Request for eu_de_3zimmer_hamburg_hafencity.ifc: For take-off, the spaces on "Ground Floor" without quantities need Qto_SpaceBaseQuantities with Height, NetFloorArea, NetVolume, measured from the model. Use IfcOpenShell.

First a look at what the model holds.

```python
import ifcopenshell
import ifcopenshell.util.element
import ifcopenshell.util.unit

model = ifcopenshell.open("eu_de_3zimmer_hamburg_hafencity.ifc")
print(model.schema)
for unit_type in ("LENGTHUNIT", "AREAUNIT", "VOLUMEUNIT"):
    print(unit_type, ifcopenshell.util.unit.calculate_unit_scale(model, unit_type))
storey = next(s for s in model.by_type("IfcBuildingStorey") if s.Name == "Ground Floor")
spaces = [e for e in ifcopenshell.util.element.get_decomposition(storey) if e.is_a("IfcSpace")]
for e in sorted(spaces, key=lambda e: e.id()):
    print(e.id(), e.is_a(), e.Name, list(ifcopenshell.util.element.get_psets(e, qtos_only=True)), sep=" | ")
```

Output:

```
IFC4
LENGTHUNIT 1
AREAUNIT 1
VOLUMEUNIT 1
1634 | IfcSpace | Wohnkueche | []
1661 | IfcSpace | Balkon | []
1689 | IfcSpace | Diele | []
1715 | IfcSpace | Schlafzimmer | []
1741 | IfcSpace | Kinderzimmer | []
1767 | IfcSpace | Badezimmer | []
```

```python
import ifcopenshell
import ifcopenshell.api.pset
import ifcopenshell.geom
import ifcopenshell.util.element
import ifcopenshell.util.shape
import ifcopenshell.util.unit

model = ifcopenshell.open("eu_de_3zimmer_hamburg_hafencity.ifc")
unit_scale = ifcopenshell.util.unit.calculate_unit_scale(model)
area_scale = ifcopenshell.util.unit.calculate_unit_scale(model, "AREAUNIT")
volume_scale = ifcopenshell.util.unit.calculate_unit_scale(model, "VOLUMEUNIT")
settings = ifcopenshell.geom.settings()

storey = next(s for s in model.by_type("IfcBuildingStorey") if s.Name == "Ground Floor")
spaces = [e for e in ifcopenshell.util.element.get_decomposition(storey) if e.is_a("IfcSpace")]

for e in sorted(spaces, key=lambda e: e.id()):
    if ifcopenshell.util.element.get_psets(e, qtos_only=True, should_inherit=False):
        continue
    # Geometry comes back in metres, in the element's own axes.
    shape = ifcopenshell.geom.create_shape(settings, e)
    values = {
        "Height": ifcopenshell.util.shape.get_z(shape.geometry) / unit_scale,
        "NetFloorArea": ifcopenshell.util.shape.get_footprint_area(shape.geometry) / area_scale,
        "NetVolume": ifcopenshell.util.shape.get_volume(shape.geometry) / volume_scale,
    }
    qto = ifcopenshell.api.pset.add_qto(model, product=e, name="Qto_SpaceBaseQuantities")
    ifcopenshell.api.pset.edit_qto(model, qto=qto, properties=values)
    print(e.id(), {k: round(v, 3) for k, v in values.items()})

model.write("eu_de_3zimmer_hamburg_hafencity_edited.ifc")
```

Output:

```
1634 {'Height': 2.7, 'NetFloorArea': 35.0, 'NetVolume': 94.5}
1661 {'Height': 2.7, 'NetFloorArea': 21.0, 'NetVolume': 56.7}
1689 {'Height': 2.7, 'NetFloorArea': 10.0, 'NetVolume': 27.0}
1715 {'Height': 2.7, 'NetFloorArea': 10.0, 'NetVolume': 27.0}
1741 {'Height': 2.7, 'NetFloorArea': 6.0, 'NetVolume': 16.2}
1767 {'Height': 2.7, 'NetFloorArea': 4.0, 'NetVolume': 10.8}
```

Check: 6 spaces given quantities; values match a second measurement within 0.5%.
